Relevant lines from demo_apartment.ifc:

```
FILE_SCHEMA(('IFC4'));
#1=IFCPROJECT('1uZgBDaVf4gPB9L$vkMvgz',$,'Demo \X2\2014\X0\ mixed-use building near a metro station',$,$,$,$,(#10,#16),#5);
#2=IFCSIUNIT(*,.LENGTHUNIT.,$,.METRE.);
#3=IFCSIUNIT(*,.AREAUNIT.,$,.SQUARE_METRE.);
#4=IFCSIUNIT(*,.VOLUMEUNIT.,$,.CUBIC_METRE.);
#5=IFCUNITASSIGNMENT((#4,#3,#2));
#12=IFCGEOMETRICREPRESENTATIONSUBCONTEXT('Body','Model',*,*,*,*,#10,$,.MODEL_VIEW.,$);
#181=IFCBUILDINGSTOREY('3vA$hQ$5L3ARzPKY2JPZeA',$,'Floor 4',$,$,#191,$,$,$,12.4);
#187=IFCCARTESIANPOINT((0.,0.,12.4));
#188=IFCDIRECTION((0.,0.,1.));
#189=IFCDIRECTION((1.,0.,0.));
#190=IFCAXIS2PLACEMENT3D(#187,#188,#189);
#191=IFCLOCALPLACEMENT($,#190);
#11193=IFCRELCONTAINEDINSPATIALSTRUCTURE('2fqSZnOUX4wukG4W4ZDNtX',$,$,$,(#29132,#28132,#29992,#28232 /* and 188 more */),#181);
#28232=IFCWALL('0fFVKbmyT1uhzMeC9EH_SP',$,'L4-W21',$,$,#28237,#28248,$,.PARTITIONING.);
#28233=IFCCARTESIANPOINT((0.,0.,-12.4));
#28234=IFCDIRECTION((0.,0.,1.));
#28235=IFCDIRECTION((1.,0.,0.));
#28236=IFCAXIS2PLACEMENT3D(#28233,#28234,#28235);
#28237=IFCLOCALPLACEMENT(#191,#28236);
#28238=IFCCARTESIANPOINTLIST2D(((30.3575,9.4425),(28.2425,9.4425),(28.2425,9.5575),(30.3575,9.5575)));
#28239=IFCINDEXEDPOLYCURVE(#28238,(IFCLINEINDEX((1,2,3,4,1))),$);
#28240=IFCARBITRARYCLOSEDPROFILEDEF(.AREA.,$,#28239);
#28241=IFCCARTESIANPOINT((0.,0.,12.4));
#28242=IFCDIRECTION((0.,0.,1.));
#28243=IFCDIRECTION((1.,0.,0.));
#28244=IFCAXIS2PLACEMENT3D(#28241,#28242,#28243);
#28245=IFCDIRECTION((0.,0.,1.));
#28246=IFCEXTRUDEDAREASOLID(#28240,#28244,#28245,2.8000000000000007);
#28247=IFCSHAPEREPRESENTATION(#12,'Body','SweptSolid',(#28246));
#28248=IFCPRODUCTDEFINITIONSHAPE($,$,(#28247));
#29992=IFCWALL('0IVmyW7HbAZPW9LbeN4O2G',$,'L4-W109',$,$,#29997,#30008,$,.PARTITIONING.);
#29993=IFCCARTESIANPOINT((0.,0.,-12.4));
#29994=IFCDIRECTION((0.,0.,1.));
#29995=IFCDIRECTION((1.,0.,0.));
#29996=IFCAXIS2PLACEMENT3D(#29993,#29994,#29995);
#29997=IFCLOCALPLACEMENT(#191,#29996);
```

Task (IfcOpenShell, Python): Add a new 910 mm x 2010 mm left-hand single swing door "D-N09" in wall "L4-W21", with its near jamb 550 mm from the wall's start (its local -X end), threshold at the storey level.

```python
import numpy as np
import ifcopenshell
import ifcopenshell.api.feature
import ifcopenshell.api.geometry
import ifcopenshell.api.root
import ifcopenshell.api.spatial
import ifcopenshell.geom
import ifcopenshell.util.element
import ifcopenshell.util.placement
import ifcopenshell.util.representation
import ifcopenshell.util.shape
import ifcopenshell.util.unit

model = ifcopenshell.open("demo_apartment.ifc")
unit_scale = ifcopenshell.util.unit.calculate_unit_scale(model)
settings = ifcopenshell.geom.settings()


def volume(element):
    """Net volume in cubic metres, openings subtracted."""
    shape = ifcopenshell.geom.create_shape(settings, element)
    return ifcopenshell.util.shape.get_volume(shape.geometry)


wall = model.by_guid("0fFVKbmyT1uhzMeC9EH_SP")
storey = ifcopenshell.util.element.get_container(wall, ifc_class="IfcBuildingStorey")
context = ifcopenshell.util.representation.get_context(model, "Model", "Body", "MODEL_VIEW")
before = volume(wall)

width, height, from_end, sill = 0.91, 2.01, 0.55, 0.0  # metres

# The wall runs along its own X axis, and the end named is its -X end.
wall_shape = ifcopenshell.geom.create_shape(settings, wall)
x, y, z = ifcopenshell.util.shape.get_vertices(wall_shape.geometry).T
start = x.min() + from_end
face, thickness = float(y.min()), float(y.max() - y.min())
wall_matrix = ifcopenshell.util.placement.get_local_placement(wall.ObjectPlacement)
level = ifcopenshell.util.placement.get_local_placement(storey.ObjectPlacement)[2, 3]


def in_wall(x, y):
    """Placement at x, y metres in the wall's axes, at sill height."""
    matrix = wall_matrix.copy()
    matrix[:, 3] = wall_matrix @ np.array([x / unit_scale, y / unit_scale, 0.0, 1.0])
    matrix[2, 3] = level + sill / unit_scale
    return matrix


# Opening: a box that overshoots both wall faces by 50 mm.
opening = ifcopenshell.api.root.create_entity(model, ifc_class="IfcOpeningElement", predefined_type="OPENING")
box = ifcopenshell.api.geometry.add_wall_representation(
    model, context=context, length=width, height=height, thickness=thickness + 0.1
)
ifcopenshell.api.geometry.assign_representation(model, product=opening, representation=box)
ifcopenshell.api.geometry.edit_object_placement(model, product=opening, matrix=in_wall(start, face - 0.05), is_si=False)
ifcopenshell.api.feature.add_feature(model, feature=opening, element=wall)

door = ifcopenshell.api.root.create_entity(model, ifc_class="IfcDoor", name="D-N09", predefined_type="DOOR")
door.OverallWidth, door.OverallHeight = width / unit_scale, height / unit_scale
door.OperationType = "SINGLE_SWING_LEFT"
body = ifcopenshell.api.geometry.add_door_representation(
    model,
    context=context,
    overall_width=door.OverallWidth,
    overall_height=door.OverallHeight,
    operation_type="SINGLE_SWING_LEFT",
    lining_properties={"LiningDepth": thickness / unit_scale, "ThresholdDepth": thickness / unit_scale},
)
ifcopenshell.api.geometry.assign_representation(model, product=door, representation=body)
ifcopenshell.api.spatial.assign_container(model, products=[door], relating_structure=storey)
ifcopenshell.api.feature.add_filling(model, opening=opening, element=door)

# The lining spans the wall, so the door starts at the wall face.
ifcopenshell.api.geometry.edit_object_placement(model, product=door, matrix=in_wall(start, face), is_si=False)

after = volume(wall)

print(f"wall volume {before:.3f} -> {after:.3f} m3")

model.write("demo_apartment_edited.ifc")
```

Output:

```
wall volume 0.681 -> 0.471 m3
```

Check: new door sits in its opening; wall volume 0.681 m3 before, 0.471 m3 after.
